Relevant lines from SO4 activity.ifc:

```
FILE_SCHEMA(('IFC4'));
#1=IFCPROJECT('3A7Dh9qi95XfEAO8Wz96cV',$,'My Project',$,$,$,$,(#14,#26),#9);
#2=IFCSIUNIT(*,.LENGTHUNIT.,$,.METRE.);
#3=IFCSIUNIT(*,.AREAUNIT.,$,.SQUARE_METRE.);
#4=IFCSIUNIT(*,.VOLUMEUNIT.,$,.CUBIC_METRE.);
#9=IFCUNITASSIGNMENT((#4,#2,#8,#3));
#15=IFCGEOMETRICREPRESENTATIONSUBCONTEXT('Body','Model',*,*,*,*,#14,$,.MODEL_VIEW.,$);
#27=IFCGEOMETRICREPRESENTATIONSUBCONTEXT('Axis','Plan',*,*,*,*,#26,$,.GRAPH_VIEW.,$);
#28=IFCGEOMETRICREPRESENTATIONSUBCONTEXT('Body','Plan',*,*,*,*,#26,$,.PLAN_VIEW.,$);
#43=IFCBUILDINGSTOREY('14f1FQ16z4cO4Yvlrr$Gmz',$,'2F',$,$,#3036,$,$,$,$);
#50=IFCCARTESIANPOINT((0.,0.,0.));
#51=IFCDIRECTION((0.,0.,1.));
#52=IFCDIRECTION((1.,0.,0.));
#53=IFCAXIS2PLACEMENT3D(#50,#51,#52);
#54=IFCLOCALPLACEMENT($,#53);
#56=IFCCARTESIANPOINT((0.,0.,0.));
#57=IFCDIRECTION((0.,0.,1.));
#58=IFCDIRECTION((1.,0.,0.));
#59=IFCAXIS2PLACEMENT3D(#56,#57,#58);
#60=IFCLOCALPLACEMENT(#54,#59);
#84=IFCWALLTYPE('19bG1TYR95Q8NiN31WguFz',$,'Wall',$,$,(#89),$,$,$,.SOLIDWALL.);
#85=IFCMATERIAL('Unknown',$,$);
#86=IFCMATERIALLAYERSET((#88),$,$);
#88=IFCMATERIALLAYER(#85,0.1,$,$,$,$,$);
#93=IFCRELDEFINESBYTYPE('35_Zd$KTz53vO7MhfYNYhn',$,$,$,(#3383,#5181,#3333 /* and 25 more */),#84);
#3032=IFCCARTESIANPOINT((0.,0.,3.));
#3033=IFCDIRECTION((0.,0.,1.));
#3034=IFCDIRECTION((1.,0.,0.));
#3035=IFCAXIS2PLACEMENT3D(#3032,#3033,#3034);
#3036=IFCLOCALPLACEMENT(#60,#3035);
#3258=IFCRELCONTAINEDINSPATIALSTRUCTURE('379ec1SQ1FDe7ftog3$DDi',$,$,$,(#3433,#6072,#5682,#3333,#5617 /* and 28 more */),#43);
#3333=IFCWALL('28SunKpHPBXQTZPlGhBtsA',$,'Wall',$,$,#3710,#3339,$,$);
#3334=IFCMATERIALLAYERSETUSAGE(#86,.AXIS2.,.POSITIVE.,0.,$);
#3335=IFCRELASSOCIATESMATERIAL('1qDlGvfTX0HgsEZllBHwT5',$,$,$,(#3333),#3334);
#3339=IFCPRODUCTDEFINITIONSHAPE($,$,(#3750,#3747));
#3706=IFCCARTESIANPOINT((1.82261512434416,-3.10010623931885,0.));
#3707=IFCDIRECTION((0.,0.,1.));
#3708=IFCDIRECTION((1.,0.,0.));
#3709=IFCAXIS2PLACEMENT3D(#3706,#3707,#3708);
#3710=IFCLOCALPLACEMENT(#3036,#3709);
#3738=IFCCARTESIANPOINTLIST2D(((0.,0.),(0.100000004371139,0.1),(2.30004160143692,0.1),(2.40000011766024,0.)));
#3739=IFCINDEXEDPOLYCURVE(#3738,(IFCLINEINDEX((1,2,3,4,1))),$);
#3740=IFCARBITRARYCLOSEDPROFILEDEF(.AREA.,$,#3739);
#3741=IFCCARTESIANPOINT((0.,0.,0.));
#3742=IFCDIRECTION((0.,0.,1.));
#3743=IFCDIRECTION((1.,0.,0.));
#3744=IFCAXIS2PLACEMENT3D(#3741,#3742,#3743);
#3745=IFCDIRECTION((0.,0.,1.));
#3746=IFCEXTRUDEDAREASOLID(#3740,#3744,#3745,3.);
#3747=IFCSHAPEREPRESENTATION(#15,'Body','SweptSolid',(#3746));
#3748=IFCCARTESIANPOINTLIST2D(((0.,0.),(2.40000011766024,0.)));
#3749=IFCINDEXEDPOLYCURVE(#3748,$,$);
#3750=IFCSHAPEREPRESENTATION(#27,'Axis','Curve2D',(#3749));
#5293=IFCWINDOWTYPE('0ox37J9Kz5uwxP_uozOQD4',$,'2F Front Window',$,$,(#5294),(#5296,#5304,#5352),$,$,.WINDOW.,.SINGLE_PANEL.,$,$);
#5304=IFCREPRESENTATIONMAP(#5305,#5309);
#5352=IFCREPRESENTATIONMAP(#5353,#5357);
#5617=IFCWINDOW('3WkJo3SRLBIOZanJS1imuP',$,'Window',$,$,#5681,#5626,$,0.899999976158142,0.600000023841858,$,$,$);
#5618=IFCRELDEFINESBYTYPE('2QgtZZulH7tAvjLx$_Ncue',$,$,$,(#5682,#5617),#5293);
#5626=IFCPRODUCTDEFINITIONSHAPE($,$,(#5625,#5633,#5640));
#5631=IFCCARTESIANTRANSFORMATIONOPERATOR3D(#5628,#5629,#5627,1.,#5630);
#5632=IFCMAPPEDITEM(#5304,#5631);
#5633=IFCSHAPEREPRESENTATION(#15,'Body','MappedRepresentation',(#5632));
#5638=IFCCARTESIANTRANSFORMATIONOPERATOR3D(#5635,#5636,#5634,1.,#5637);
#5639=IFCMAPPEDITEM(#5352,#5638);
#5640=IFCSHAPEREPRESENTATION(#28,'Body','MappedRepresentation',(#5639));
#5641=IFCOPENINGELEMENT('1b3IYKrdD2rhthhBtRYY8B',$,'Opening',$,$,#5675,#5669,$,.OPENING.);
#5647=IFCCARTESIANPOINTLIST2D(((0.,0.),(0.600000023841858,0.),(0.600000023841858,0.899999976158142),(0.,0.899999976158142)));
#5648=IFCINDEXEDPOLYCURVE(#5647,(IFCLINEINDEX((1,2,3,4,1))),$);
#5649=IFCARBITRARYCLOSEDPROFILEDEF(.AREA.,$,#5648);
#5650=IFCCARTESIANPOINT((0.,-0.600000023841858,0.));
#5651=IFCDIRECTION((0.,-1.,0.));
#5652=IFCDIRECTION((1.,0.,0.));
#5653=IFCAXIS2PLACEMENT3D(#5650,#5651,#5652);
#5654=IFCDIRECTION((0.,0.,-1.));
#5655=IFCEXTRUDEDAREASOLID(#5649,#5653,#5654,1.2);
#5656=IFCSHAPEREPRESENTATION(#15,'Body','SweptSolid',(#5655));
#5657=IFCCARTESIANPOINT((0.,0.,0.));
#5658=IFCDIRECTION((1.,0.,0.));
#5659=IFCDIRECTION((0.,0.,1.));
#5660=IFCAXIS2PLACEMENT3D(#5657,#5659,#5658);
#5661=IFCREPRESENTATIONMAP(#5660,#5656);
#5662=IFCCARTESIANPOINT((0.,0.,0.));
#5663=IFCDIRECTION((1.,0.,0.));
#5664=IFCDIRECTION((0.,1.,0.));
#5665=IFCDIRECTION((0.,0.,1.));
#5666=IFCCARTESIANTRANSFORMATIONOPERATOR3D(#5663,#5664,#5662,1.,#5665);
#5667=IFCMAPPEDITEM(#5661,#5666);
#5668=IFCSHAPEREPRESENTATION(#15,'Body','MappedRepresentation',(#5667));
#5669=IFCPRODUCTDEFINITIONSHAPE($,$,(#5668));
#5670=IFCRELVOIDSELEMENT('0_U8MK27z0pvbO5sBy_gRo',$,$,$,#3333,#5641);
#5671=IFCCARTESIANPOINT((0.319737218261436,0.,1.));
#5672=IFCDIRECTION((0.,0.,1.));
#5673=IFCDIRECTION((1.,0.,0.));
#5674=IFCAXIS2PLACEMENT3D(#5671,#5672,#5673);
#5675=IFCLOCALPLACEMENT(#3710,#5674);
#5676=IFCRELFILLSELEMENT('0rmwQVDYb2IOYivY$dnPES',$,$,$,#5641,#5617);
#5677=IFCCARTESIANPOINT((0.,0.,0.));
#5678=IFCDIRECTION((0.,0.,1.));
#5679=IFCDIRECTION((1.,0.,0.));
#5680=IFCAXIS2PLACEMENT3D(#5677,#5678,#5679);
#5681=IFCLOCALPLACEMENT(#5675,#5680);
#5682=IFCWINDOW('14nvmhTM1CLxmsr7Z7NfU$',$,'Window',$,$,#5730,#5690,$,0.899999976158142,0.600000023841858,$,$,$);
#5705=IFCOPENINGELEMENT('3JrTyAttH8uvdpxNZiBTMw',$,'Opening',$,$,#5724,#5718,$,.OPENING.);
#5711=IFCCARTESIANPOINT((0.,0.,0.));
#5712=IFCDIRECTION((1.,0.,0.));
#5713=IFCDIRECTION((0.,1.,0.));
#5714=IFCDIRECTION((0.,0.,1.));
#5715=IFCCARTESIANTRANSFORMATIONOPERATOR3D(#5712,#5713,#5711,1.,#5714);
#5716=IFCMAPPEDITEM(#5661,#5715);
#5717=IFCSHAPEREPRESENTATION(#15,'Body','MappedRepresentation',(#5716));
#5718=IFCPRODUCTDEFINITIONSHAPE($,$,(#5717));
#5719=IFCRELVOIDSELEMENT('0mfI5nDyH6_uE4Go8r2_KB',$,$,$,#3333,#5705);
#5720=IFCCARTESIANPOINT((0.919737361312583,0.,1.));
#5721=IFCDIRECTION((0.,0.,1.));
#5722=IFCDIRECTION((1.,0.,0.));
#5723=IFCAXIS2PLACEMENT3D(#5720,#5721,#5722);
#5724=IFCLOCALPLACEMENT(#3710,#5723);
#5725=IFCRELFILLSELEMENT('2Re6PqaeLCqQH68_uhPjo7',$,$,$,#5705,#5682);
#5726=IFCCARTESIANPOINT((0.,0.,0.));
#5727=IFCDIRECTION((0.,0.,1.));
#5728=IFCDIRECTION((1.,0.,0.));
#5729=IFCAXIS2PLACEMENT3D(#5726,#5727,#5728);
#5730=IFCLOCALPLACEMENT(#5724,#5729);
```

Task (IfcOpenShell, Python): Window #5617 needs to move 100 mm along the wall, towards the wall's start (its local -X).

```python
import ifcopenshell
import ifcopenshell.api.geometry
import ifcopenshell.util.placement
import ifcopenshell.util.unit

model = ifcopenshell.open("SO4 activity.ifc")
unit_scale = ifcopenshell.util.unit.calculate_unit_scale(model)

window = model.by_guid("3WkJo3SRLBIOZanJS1imuP")
opening = window.FillsVoids[0].RelatingOpeningElement
wall = opening.VoidsElements[0].RelatingBuildingElement

wall_matrix = ifcopenshell.util.placement.get_local_placement(wall.ObjectPlacement)
shift = wall_matrix[:3, 0] * -0.1 / unit_scale
before = ifcopenshell.util.placement.get_local_placement(window.ObjectPlacement)[:3, 3].copy()

# The window is placed relative to its opening, so it follows when the opening moves.
matrix = ifcopenshell.util.placement.get_local_placement(opening.ObjectPlacement)
matrix[:3, 3] += shift
ifcopenshell.api.geometry.edit_object_placement(
    model, product=opening, matrix=matrix, is_si=False, should_transform_children=True
)

after = ifcopenshell.util.placement.get_local_placement(window.ObjectPlacement)[:3, 3]
print("window moved by", (after - before).round(3) + 0.0)

model.write("SO4 activity_edited.ifc")
```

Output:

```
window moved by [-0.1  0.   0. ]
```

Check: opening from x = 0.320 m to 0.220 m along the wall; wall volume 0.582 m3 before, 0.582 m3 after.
